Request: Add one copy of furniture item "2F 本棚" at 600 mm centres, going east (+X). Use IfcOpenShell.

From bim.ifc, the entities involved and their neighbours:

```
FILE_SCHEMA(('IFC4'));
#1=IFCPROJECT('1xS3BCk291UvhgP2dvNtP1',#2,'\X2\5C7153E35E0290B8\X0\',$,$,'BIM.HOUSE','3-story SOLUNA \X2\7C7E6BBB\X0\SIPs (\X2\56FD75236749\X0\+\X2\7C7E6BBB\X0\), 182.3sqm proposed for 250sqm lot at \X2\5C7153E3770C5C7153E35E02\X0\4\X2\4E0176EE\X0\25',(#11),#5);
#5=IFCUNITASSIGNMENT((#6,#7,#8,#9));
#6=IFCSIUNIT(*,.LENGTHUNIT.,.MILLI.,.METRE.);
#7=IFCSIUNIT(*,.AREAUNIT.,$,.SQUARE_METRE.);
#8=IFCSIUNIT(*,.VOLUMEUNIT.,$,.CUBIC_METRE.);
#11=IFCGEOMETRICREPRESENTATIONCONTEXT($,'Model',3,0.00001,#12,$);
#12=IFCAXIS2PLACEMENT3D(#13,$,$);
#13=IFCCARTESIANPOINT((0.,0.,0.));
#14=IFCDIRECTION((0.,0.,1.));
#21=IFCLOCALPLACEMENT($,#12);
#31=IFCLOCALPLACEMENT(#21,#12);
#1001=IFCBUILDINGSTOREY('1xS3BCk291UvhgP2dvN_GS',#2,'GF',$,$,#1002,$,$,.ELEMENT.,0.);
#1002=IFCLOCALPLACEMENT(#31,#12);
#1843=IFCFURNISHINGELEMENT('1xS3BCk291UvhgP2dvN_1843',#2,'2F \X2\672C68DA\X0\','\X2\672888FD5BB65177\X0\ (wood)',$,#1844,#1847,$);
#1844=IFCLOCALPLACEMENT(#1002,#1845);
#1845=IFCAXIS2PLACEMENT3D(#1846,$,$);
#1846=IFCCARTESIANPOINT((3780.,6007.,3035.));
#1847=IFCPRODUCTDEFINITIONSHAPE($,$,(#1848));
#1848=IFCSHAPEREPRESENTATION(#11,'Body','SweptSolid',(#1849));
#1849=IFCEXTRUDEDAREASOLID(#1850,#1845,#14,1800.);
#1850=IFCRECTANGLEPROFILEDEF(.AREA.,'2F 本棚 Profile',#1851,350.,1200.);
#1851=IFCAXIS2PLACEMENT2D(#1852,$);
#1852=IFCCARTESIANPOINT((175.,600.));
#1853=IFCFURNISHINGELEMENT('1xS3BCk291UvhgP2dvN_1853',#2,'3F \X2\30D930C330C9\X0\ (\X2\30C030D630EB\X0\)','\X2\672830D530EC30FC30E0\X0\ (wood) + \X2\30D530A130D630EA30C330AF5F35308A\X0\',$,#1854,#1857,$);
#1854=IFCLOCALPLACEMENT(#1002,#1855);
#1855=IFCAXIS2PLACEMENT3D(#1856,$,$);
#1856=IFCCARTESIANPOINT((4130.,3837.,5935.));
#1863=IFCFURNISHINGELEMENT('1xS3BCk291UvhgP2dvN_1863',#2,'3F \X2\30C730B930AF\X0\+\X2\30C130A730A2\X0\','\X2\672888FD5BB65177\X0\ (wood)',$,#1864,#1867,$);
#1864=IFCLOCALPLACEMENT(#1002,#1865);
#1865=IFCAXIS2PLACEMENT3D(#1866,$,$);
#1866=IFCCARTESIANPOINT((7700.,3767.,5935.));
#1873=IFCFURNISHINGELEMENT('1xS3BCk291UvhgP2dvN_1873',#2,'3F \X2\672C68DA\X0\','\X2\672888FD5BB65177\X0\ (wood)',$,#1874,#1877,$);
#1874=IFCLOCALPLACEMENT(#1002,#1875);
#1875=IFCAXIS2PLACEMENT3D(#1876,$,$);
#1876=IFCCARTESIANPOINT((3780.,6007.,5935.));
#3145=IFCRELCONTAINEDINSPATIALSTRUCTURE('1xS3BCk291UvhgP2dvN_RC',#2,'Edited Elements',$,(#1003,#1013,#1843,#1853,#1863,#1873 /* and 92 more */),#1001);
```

```python
import numpy as np
import ifcopenshell
import ifcopenshell.api.geometry
import ifcopenshell.api.root
import ifcopenshell.util.element
import ifcopenshell.util.placement
import ifcopenshell.util.unit

model = ifcopenshell.open("bim.ifc")
unit_scale = ifcopenshell.util.unit.calculate_unit_scale(model)


def reuse_history(source, copy):
    """copy_class also copies each property set's owner history, people and application; keep the originals."""
    for rel in copy.IsDefinedBy:
        if rel.is_a("IfcRelDefinesByProperties") and (history := rel.RelatingPropertyDefinition.OwnerHistory):
            rel.RelatingPropertyDefinition.OwnerHistory = source.OwnerHistory
            ifcopenshell.util.element.remove_deep2(model, history)


source = model.by_guid("1xS3BCk291UvhgP2dvN_1843")
base = ifcopenshell.util.placement.get_local_placement(source.ObjectPlacement)
step = np.array([1.0, 0.0, 0.0]) * 0.6 / unit_scale

for i in range(1, 2):
    copy = ifcopenshell.api.root.copy_class(model, product=source)
    copy.Representation = ifcopenshell.util.element.copy_deep(
        model, source.Representation, exclude=["IfcGeometricRepresentationContext", "IfcRepresentationMap"]
    )
    reuse_history(source, copy)
    matrix = base.copy()
    matrix[:3, 3] += i * step
    print("added at", matrix[:3, 3].round(3) + 0.0)
    ifcopenshell.api.geometry.edit_object_placement(model, product=copy, matrix=matrix, is_si=False)

model.write("bim_edited.ifc")
```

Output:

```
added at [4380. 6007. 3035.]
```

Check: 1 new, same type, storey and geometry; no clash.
